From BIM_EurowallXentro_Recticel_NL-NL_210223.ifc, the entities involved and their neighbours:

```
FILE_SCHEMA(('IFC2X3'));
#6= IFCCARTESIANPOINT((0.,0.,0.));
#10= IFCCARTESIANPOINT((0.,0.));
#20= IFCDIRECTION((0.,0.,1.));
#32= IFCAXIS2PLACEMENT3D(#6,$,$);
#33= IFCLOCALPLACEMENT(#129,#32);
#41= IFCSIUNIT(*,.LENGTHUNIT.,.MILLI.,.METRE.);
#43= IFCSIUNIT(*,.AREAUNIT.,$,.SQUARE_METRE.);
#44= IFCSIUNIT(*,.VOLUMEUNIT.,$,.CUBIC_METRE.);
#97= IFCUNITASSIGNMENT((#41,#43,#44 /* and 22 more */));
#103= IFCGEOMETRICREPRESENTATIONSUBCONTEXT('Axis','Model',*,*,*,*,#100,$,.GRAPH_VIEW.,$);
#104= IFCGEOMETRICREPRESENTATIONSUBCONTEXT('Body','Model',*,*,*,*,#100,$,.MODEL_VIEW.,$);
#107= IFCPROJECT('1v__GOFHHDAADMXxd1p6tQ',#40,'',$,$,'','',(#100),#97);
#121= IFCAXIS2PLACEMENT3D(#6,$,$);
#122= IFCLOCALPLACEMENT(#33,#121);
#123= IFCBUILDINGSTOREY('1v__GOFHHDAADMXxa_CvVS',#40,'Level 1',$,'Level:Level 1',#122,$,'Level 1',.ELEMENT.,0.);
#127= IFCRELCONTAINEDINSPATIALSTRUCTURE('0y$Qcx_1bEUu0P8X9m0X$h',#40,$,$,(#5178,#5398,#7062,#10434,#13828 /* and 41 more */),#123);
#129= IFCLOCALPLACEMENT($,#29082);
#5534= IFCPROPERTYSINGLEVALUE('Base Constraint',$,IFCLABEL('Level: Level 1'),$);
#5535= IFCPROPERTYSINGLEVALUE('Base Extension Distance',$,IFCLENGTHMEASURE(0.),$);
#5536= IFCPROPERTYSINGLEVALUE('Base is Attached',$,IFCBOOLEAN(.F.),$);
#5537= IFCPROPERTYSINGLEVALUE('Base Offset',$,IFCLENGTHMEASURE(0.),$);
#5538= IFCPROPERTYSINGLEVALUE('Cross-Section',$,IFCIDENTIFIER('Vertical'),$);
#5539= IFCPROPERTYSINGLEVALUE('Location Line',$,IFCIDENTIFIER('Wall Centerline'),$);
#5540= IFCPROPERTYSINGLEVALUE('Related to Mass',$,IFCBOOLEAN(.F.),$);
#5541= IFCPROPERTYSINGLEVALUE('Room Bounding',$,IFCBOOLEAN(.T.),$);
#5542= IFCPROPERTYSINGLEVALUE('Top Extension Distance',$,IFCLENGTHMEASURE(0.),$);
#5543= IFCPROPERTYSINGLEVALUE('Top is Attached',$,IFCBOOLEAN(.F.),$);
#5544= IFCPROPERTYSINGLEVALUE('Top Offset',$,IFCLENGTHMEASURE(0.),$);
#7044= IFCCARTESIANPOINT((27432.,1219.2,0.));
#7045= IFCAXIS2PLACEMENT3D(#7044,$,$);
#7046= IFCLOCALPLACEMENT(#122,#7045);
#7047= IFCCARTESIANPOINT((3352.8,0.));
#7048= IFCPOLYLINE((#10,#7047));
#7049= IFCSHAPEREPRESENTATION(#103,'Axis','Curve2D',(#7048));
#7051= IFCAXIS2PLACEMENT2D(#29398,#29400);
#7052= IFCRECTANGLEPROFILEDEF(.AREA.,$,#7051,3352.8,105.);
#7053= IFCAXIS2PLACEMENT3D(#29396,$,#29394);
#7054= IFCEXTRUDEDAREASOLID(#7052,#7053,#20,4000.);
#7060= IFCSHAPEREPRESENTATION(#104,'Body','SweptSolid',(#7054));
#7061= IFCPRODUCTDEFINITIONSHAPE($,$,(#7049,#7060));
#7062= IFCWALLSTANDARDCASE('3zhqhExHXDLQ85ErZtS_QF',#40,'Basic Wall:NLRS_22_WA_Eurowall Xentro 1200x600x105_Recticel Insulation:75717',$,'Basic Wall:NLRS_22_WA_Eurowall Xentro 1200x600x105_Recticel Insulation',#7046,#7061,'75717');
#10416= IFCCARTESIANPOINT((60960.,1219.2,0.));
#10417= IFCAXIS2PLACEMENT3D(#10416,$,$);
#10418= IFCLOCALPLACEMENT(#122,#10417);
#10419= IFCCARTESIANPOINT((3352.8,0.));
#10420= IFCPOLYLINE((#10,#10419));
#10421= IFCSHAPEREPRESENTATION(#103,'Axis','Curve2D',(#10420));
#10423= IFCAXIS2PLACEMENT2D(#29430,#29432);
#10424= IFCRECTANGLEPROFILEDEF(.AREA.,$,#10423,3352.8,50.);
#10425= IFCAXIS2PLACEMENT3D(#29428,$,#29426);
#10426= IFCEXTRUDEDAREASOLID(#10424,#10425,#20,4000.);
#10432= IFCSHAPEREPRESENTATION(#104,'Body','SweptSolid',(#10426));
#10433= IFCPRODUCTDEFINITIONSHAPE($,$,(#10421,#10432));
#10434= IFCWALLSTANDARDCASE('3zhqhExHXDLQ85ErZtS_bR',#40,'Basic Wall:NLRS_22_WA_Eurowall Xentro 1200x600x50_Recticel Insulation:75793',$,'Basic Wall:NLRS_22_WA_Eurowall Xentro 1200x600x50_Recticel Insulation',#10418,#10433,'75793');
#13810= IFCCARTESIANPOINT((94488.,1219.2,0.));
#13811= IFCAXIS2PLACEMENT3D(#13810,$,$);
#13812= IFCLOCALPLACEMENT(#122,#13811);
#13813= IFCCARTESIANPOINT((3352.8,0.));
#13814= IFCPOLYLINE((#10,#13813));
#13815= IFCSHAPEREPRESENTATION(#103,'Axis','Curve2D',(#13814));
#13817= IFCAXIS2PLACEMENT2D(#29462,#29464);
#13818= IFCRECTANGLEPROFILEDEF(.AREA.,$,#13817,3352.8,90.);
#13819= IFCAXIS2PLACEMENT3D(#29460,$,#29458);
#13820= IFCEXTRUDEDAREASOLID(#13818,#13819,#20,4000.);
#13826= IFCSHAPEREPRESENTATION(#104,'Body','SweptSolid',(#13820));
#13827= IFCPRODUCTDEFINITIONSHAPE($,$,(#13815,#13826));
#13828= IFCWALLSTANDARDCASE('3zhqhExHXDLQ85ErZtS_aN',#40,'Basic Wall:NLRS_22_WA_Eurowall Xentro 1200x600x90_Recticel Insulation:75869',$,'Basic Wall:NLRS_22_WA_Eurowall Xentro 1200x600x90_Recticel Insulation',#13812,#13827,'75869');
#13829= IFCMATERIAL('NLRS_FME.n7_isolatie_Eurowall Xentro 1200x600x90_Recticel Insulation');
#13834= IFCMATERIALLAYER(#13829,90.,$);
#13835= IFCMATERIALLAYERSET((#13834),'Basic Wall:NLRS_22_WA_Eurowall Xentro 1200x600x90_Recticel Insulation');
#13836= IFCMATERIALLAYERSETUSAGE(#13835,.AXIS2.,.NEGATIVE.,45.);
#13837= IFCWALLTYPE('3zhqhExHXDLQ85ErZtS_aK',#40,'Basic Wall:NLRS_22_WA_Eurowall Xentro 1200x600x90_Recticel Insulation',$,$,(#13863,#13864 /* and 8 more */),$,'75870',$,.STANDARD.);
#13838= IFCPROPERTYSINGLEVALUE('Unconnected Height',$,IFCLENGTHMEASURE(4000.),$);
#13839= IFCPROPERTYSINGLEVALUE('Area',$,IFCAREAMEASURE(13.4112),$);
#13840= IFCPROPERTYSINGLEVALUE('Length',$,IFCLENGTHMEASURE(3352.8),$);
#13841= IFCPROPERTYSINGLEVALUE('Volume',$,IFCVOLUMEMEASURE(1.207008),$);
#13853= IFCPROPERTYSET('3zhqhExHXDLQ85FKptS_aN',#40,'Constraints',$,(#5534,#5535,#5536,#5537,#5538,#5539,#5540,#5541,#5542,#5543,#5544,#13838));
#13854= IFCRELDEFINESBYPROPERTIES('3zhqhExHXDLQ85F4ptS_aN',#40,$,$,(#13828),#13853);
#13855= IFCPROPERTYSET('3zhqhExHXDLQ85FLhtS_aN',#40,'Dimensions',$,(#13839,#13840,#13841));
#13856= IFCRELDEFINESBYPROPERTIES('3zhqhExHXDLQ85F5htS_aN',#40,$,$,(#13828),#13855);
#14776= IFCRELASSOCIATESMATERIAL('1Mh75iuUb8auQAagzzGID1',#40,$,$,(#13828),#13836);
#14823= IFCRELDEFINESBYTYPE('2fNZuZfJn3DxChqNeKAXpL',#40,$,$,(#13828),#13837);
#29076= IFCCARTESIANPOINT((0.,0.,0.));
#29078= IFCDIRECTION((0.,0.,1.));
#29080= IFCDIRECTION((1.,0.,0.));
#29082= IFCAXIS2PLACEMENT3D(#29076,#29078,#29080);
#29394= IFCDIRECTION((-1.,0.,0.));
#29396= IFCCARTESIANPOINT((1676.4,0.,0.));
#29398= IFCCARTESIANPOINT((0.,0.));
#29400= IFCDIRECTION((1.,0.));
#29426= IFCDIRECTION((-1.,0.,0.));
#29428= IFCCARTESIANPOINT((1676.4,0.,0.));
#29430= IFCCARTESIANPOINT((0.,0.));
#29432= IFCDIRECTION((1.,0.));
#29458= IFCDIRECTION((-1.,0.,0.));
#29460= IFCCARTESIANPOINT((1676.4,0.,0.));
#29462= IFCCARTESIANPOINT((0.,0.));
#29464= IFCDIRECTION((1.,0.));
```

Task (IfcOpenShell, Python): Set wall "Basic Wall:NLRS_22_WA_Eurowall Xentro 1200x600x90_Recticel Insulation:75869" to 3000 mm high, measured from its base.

```python
import ifcopenshell
import ifcopenshell.api.pset
import ifcopenshell.geom
import ifcopenshell.util.element
import ifcopenshell.util.representation
import ifcopenshell.util.shape
import ifcopenshell.util.unit

model = ifcopenshell.open("BIM_EurowallXentro_Recticel_NL-NL_210223.ifc")
unit_scale = ifcopenshell.util.unit.calculate_unit_scale(model)
area_scale = ifcopenshell.util.unit.calculate_unit_scale(model, "AREAUNIT")
volume_scale = ifcopenshell.util.unit.calculate_unit_scale(model, "VOLUMEUNIT")
settings = ifcopenshell.geom.settings()


def volume(element):
    """Net volume in cubic metres, openings subtracted."""
    shape = ifcopenshell.geom.create_shape(settings, element)
    return ifcopenshell.util.shape.get_volume(shape.geometry)


wall = model.by_id(13828)
before = volume(wall)

body = ifcopenshell.util.representation.get_representation(wall, "Model", "Body")
solid = body.Items[0]
old_height = solid.Depth
solid.Depth = 3 / unit_scale
after = volume(wall)
thickness = 0.09  # wall thickness in metres

# Update the stored height, areas and volumes.
pset = model.by_id(ifcopenshell.util.element.get_pset(wall, "Constraints", should_inherit=False)["id"])
ifcopenshell.api.pset.edit_pset(model, pset=pset, properties={
    "Unconnected Height": model.create_entity("IfcLengthMeasure", solid.Depth),
})
pset = model.by_id(ifcopenshell.util.element.get_pset(wall, "Dimensions", should_inherit=False)["id"])
ifcopenshell.api.pset.edit_pset(model, pset=pset, properties={
    "Area": model.create_entity("IfcAreaMeasure", after / thickness / area_scale),
    "Volume": model.create_entity("IfcVolumeMeasure", after / volume_scale),
})

print(f"height {old_height:g} -> {solid.Depth:g}, volume {before:.3f} -> {after:.3f} m3")

model.write("BIM_EurowallXentro_Recticel_NL-NL_210223_v2.ifc")
```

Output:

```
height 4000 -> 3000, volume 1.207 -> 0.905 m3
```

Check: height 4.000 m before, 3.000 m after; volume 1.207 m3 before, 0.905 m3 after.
